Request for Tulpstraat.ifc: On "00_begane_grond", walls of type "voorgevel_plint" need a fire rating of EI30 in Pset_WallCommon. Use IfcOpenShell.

First a look at what the model holds.

```python
import ifcopenshell
import ifcopenshell.util.element

model = ifcopenshell.open("Tulpstraat.ifc")
print(model.schema)
storey = next(s for s in model.by_type("IfcBuildingStorey") if s.Name == "00_begane_grond")
walls = [e for e in ifcopenshell.util.element.get_decomposition(storey) if e.is_a("IfcWall")]
seen = {}
for e in walls:
    element_type = ifcopenshell.util.element.get_type(e)
    key = (element_type.Name if element_type != e and element_type else None, ifcopenshell.util.element.get_pset(e, "Pset_WallCommon", "FireRating"))
    seen[key] = seen.get(key, 0) + 1
for (name, value), count in sorted(seen.items(), key=str):
    print(count, "x", name, "|", value)
```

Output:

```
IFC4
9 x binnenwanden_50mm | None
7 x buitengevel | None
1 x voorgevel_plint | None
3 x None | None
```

```python
import ifcopenshell
import ifcopenshell.api.pset
import ifcopenshell.util.element

model = ifcopenshell.open("Tulpstraat.ifc")

storey = next(s for s in model.by_type("IfcBuildingStorey") if s.Name == "00_begane_grond")
walls = [e for e in ifcopenshell.util.element.get_decomposition(storey) if e.is_a("IfcWall")]

count = 0
for e in walls:
    element_type = ifcopenshell.util.element.get_type(e)
    if element_type in (None, e) or element_type.Name != "voorgevel_plint":
        continue
    # add_pset returns the element's existing set when there is one.
    pset = ifcopenshell.api.pset.add_pset(model, product=e, name="Pset_WallCommon")
    ifcopenshell.api.pset.edit_pset(model, pset=pset, properties={"FireRating": "EI30"})
    count += 1

print(count, "walls updated")

model.write("Tulpstraat_rev.ifc")
```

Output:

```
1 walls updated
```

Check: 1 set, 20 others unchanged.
